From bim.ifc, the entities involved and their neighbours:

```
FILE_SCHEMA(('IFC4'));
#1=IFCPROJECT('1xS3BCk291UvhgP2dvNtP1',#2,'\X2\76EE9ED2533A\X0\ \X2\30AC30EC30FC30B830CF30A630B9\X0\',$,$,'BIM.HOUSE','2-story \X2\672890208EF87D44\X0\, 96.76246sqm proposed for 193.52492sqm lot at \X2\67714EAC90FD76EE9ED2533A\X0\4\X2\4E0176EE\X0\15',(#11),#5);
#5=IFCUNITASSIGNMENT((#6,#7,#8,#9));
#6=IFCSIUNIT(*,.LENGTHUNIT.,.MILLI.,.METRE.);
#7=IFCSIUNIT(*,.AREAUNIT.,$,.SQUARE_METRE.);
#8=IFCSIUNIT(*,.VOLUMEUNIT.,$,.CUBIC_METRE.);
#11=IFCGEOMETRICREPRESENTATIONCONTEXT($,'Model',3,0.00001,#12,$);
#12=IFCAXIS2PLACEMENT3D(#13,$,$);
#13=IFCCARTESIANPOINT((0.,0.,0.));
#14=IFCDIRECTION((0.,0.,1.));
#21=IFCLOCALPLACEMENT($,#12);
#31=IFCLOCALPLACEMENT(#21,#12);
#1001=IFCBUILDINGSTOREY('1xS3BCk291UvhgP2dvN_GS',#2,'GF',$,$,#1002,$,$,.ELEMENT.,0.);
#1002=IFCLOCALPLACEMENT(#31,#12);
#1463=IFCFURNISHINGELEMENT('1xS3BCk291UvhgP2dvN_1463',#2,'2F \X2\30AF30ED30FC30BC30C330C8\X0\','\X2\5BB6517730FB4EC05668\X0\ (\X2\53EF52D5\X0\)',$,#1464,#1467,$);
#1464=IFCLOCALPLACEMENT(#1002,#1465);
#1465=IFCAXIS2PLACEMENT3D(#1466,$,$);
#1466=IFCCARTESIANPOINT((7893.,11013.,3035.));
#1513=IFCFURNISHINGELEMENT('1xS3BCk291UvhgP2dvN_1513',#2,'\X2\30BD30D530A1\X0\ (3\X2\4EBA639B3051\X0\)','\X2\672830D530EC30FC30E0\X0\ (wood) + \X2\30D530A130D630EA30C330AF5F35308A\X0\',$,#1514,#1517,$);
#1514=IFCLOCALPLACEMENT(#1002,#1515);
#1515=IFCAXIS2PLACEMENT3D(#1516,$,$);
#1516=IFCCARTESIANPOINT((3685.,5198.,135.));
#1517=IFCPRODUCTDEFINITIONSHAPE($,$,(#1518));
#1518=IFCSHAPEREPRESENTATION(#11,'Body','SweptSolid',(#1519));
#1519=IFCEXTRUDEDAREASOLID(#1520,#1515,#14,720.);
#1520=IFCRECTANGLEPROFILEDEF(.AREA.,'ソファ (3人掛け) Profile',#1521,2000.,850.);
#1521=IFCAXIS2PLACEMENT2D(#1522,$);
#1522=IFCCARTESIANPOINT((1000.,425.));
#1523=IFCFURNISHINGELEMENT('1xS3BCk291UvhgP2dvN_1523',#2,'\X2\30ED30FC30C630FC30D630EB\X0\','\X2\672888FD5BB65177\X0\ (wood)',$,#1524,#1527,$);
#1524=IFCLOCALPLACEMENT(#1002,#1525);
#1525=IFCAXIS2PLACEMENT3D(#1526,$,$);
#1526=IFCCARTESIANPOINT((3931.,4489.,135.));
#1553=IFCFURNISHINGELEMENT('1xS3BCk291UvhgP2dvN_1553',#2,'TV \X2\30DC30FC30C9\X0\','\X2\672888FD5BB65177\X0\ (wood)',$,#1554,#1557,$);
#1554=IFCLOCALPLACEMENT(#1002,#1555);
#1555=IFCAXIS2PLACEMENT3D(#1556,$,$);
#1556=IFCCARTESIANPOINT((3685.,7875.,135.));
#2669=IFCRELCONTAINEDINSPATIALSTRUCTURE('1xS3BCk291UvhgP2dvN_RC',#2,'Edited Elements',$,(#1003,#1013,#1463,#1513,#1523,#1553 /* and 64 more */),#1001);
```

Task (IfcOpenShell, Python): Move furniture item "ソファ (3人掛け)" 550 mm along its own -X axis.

```python
import ifcopenshell
import ifcopenshell.api.geometry
import ifcopenshell.util.placement
import ifcopenshell.util.unit

model = ifcopenshell.open("bim.ifc")
unit_scale = ifcopenshell.util.unit.calculate_unit_scale(model)

item = model.by_guid("1xS3BCk291UvhgP2dvN_1513")
matrix = ifcopenshell.util.placement.get_local_placement(item.ObjectPlacement)
matrix[:3, 3] -= matrix[:3, 0] * 0.55 / unit_scale
ifcopenshell.api.geometry.edit_object_placement(model, product=item, matrix=matrix, is_si=False)

print(ifcopenshell.util.placement.get_local_placement(item.ObjectPlacement).round(3) + 0.0)

model.write("bim-out.ifc")
```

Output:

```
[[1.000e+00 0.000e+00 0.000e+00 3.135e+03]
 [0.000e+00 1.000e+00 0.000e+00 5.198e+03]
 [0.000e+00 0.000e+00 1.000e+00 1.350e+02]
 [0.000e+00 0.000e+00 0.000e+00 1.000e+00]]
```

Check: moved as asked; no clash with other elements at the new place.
